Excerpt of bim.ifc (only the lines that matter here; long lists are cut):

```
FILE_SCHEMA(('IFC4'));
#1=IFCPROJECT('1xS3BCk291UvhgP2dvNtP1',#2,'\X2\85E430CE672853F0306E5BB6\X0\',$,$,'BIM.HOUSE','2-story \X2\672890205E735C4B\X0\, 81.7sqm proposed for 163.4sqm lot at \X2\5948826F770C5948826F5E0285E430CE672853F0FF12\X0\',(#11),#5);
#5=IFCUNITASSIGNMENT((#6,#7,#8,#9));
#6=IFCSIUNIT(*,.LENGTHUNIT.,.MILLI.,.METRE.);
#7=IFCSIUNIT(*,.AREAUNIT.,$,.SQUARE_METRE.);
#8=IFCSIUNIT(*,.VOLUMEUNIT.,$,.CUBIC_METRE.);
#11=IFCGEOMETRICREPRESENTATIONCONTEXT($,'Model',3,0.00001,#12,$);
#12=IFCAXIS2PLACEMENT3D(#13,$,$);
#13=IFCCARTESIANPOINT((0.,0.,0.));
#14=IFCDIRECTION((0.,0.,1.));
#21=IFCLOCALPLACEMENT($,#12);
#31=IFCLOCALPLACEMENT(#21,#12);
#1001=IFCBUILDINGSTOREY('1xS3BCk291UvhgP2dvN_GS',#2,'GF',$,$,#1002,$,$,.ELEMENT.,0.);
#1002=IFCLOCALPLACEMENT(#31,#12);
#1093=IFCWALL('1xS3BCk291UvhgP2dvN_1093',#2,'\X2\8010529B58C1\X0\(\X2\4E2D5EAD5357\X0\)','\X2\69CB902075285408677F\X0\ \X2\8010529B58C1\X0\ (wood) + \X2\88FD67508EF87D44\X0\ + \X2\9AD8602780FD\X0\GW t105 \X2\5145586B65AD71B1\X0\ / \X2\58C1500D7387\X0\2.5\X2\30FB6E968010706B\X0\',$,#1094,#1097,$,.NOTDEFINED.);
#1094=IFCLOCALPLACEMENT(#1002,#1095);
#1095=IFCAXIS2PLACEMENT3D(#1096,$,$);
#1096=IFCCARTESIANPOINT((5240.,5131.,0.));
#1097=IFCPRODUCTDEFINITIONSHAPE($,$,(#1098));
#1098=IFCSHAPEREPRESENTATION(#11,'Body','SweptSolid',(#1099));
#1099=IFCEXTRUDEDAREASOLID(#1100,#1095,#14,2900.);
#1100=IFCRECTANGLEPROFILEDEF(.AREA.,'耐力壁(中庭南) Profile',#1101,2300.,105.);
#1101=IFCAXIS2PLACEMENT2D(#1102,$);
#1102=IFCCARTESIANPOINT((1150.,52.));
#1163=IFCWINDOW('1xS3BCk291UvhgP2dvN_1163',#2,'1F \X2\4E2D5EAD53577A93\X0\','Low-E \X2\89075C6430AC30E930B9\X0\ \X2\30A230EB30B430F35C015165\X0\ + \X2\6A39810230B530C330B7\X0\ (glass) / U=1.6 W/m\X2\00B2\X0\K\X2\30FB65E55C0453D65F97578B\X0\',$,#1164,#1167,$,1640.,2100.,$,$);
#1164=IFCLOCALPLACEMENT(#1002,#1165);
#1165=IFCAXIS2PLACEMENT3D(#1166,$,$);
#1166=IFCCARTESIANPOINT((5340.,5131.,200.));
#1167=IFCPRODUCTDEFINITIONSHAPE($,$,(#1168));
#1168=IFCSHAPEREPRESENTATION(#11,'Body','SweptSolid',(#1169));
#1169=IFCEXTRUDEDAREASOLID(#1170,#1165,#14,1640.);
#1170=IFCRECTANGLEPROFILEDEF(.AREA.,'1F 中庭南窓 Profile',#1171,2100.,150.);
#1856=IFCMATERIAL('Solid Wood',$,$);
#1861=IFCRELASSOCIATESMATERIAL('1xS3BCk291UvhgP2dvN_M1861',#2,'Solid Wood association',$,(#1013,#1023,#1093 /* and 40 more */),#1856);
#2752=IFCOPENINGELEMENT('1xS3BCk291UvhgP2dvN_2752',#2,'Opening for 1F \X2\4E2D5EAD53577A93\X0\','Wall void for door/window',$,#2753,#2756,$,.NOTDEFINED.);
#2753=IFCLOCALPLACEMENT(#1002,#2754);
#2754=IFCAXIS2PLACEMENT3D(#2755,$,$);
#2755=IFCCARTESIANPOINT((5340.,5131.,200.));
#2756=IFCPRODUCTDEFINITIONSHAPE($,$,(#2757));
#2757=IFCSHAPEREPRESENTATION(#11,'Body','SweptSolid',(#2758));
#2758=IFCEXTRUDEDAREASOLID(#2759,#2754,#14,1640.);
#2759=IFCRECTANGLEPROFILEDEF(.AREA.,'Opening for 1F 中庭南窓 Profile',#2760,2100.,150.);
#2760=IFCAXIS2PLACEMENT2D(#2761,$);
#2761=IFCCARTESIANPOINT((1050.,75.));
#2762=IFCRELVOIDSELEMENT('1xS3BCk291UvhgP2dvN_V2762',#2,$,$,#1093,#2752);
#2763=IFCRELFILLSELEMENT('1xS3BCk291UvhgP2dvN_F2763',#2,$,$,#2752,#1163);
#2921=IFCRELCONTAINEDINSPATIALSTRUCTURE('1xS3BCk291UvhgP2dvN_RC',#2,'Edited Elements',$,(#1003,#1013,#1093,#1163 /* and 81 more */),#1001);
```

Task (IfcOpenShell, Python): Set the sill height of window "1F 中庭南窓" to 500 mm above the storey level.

```python
import numpy as np
import ifcopenshell
import ifcopenshell.api.geometry
import ifcopenshell.geom
import ifcopenshell.util.element
import ifcopenshell.util.placement
import ifcopenshell.util.shape
import ifcopenshell.util.unit

model = ifcopenshell.open("bim.ifc")
unit_scale = ifcopenshell.util.unit.calculate_unit_scale(model)

window = model.by_id(1163)
opening = window.FillsVoids[0].RelatingOpeningElement
storey = ifcopenshell.util.element.get_container(window, ifc_class="IfcBuildingStorey")
level = ifcopenshell.util.placement.get_local_placement(storey.ObjectPlacement)[2, 3]

# The opening's origin need not be at the sill, so measure its lowest point.
shape = ifcopenshell.geom.create_shape(ifcopenshell.geom.settings(), opening)
bottom = ifcopenshell.util.shape.get_shape_bottom_elevation(shape, shape.geometry) / unit_scale
dz = level + 500.0 - bottom

shift = np.array([0.0, 0.0, dz])
# The window is not placed relative to its opening, so move both.
for product in (opening, window):
    matrix = ifcopenshell.util.placement.get_local_placement(product.ObjectPlacement)
    matrix[:3, 3] += shift
    ifcopenshell.api.geometry.edit_object_placement(model, product=product, matrix=matrix, is_si=False)

print(f"moved by {dz * unit_scale:+.3f} m")

model.write("bim_updated.ifc")
```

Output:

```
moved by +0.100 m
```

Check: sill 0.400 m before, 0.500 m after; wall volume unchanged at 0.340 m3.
